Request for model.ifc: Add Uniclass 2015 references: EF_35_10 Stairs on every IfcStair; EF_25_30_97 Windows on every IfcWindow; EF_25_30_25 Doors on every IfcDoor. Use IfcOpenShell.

First a look at what the model holds.

```python
import ifcopenshell

model = ifcopenshell.open("model.ifc")
print(model.schema)
print("classifications:", [c.Name for c in model.by_type("IfcClassification")])
for ifc_class in ("IfcDoor", "IfcRoof", "IfcStair", "IfcWall", "IfcWindow"):
    print(ifc_class, len(model.by_type(ifc_class)))
```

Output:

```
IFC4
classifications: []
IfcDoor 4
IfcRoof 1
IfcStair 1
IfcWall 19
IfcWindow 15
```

```python
import ifcopenshell
import ifcopenshell.api.classification

model = ifcopenshell.open("model.ifc")

system = ifcopenshell.api.classification.add_classification(model, classification="Uniclass 2015")

codes = {
    "IfcStair": ("EF_35_10", "Stairs"),
    "IfcWindow": ("EF_25_30_97", "Windows"),
    "IfcDoor": ("EF_25_30_25", "Doors"),
}
for ifc_class, (code, name) in codes.items():
    products = model.by_type(ifc_class)
    ifcopenshell.api.classification.add_reference(
        model, products=products, classification=system, identification=code, name=name
    )
    print(code, len(products))

model.write("model_v2.ifc")
```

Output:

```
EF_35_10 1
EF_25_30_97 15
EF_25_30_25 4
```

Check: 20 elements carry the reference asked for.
